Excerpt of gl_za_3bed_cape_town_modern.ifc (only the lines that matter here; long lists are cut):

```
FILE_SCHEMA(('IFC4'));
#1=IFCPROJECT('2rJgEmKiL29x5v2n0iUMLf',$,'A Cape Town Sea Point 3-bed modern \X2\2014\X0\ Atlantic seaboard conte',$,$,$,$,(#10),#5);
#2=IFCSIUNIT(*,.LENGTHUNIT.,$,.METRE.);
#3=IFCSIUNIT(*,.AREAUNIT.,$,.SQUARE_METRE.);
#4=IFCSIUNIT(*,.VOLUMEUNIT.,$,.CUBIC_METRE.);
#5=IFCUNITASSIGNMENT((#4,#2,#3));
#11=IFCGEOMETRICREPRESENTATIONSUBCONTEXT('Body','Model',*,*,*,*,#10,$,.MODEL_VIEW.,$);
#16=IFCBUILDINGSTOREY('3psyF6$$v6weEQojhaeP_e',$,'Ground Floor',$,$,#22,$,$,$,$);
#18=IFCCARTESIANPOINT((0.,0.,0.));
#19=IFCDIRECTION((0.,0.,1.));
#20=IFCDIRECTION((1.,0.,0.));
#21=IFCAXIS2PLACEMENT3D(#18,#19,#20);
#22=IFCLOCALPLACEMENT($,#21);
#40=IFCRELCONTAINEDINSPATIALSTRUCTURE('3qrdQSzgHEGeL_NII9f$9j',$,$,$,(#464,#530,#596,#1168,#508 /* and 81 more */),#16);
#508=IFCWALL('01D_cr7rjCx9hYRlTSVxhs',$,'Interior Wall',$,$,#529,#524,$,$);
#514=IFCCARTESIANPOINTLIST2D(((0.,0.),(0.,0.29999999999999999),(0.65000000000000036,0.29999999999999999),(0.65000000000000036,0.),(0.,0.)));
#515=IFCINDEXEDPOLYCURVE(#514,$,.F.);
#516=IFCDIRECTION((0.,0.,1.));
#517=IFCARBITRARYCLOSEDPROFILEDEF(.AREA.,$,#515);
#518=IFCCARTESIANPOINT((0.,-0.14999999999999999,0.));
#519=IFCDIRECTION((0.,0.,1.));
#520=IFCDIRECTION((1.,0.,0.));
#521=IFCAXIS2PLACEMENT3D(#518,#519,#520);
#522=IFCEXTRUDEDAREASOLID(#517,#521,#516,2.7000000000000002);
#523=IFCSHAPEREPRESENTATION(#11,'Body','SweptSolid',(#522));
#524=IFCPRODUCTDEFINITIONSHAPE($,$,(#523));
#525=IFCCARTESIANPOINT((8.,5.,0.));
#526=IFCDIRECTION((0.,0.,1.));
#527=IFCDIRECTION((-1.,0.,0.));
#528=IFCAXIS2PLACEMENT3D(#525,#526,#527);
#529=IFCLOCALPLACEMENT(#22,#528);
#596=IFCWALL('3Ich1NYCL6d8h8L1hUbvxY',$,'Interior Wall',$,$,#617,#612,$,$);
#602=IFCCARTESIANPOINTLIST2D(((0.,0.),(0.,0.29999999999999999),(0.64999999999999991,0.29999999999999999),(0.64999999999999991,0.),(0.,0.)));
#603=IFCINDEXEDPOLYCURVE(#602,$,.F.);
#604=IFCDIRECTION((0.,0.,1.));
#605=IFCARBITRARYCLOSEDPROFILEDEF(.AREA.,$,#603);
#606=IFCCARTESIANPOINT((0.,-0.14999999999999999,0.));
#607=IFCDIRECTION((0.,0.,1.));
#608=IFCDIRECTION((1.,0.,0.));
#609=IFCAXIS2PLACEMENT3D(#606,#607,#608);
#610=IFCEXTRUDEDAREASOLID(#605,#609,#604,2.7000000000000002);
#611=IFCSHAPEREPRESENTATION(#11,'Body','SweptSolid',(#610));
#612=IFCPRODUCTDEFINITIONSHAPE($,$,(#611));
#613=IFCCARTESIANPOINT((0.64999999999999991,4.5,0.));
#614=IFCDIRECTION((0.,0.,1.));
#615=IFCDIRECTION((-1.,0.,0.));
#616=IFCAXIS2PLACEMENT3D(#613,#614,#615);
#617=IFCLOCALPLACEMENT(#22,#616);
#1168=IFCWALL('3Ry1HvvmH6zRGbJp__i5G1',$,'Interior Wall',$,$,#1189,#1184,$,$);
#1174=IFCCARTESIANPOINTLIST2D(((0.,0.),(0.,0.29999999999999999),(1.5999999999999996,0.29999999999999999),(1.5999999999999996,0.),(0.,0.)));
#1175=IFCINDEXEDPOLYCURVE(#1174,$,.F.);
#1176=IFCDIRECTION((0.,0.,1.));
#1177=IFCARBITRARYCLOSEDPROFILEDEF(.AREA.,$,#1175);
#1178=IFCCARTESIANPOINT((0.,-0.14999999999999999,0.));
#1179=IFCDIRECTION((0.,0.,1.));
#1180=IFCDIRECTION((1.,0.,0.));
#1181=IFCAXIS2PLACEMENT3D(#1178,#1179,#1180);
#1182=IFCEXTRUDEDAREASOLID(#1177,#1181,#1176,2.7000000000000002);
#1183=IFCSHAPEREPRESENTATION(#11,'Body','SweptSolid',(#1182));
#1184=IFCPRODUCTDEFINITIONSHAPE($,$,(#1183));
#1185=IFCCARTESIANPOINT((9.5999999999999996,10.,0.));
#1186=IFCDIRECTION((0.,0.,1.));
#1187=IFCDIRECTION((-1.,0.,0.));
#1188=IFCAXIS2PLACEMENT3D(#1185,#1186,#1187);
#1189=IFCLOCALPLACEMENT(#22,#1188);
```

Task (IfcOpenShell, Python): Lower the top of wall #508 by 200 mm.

```python
import ifcopenshell
import ifcopenshell.geom
import ifcopenshell.util.representation
import ifcopenshell.util.shape

model = ifcopenshell.open("gl_za_3bed_cape_town_modern.ifc")
settings = ifcopenshell.geom.settings()


def volume(element):
    """Net volume in cubic metres, openings subtracted."""
    shape = ifcopenshell.geom.create_shape(settings, element)
    return ifcopenshell.util.shape.get_volume(shape.geometry)


wall = model.by_guid("01D_cr7rjCx9hYRlTSVxhs")
before = volume(wall)

body = ifcopenshell.util.representation.get_representation(wall, "Model", "Body")
solid = body.Items[0]
old_height = solid.Depth
solid.Depth -= 0.2
after = volume(wall)

print(f"height {old_height:g} -> {solid.Depth:g}, volume {before:.3f} -> {after:.3f} m3")

model.write("gl_za_3bed_cape_town_modern_updated.ifc")
```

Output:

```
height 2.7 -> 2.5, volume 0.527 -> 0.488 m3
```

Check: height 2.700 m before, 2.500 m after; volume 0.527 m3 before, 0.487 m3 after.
